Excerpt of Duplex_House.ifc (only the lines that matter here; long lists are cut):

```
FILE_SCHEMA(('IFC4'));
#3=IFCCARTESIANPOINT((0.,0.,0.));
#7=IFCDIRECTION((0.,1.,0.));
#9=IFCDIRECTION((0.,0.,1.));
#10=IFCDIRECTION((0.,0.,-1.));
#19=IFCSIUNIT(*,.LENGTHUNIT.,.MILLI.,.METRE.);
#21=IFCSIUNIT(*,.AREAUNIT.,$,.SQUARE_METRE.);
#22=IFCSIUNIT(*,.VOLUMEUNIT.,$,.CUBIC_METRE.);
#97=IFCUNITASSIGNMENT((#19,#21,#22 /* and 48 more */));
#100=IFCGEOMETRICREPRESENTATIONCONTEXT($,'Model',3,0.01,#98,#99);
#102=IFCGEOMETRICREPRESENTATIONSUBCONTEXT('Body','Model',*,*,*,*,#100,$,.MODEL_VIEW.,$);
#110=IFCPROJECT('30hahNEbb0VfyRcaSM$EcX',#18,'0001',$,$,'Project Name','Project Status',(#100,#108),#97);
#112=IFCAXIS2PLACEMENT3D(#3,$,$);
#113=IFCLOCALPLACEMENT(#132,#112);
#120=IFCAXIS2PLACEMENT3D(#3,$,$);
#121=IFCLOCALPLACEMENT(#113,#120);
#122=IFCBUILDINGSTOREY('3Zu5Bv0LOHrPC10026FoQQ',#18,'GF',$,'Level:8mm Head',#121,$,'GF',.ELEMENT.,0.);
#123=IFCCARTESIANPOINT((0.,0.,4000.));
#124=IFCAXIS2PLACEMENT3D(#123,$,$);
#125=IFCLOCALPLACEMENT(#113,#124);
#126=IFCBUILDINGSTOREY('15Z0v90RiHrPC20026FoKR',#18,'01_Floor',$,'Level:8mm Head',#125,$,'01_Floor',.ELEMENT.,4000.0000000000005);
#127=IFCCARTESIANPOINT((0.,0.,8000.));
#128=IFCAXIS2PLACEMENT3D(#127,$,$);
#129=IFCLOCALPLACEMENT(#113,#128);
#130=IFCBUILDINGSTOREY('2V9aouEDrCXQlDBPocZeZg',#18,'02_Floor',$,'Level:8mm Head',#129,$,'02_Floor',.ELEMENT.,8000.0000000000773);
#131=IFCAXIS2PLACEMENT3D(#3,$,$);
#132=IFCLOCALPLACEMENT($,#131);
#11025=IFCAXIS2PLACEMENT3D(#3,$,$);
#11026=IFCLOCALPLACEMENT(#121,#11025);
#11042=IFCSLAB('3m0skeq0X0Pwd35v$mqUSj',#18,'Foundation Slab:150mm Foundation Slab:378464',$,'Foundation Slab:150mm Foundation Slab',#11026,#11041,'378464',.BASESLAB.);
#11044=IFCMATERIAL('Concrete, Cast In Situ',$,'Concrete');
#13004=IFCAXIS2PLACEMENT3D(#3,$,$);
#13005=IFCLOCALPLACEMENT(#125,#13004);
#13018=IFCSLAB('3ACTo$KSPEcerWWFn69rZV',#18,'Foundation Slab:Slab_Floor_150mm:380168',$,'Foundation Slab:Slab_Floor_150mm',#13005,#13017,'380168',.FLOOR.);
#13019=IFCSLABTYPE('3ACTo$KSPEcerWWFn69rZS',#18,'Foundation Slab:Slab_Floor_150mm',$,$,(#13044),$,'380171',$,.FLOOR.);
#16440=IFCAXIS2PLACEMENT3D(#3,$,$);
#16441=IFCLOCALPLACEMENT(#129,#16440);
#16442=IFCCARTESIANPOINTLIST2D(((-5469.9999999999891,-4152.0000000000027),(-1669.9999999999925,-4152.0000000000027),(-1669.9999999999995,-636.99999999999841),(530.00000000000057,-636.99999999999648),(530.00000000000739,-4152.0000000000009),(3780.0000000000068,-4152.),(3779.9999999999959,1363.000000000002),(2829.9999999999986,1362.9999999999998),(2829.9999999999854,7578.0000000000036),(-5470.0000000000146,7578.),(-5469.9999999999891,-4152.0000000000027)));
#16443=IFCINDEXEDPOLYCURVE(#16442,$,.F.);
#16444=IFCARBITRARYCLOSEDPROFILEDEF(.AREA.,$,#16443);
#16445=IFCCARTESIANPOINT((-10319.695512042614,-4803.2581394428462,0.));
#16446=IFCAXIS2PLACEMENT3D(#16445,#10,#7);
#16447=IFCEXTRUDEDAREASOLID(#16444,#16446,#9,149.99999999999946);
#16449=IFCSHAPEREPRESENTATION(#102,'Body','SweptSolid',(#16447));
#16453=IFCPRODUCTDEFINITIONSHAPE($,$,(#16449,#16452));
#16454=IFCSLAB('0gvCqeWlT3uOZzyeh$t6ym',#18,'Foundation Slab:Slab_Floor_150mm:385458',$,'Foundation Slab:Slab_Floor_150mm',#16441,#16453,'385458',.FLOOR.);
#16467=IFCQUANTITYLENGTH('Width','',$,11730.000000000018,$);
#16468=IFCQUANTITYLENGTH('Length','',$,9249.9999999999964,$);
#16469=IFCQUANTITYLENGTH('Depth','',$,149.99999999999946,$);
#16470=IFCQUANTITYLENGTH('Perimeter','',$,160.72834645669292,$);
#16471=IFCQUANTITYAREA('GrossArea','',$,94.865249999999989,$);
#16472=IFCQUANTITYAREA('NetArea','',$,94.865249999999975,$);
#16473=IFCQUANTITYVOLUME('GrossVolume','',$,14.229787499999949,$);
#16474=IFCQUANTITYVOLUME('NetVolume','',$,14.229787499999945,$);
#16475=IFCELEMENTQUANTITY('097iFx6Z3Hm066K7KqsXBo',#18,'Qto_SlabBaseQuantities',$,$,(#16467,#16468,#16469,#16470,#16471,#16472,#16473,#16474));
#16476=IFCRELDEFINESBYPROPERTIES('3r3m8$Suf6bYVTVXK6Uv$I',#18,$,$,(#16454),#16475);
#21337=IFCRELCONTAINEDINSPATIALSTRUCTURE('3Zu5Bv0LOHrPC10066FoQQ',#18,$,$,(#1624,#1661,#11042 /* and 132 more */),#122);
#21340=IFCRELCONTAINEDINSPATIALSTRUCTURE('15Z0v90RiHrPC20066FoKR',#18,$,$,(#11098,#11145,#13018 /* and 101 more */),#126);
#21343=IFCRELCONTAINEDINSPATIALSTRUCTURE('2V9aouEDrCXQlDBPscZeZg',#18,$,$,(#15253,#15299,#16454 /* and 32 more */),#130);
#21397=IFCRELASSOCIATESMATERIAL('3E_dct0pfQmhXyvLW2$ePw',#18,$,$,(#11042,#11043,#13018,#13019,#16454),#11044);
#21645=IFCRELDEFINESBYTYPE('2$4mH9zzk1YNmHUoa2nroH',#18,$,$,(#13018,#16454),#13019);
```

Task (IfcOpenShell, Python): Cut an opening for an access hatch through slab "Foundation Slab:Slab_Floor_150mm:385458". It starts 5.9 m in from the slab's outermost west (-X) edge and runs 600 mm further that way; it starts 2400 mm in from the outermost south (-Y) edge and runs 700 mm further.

```python
import numpy as np
import ifcopenshell
import ifcopenshell.api.feature
import ifcopenshell.api.geometry
import ifcopenshell.api.pset
import ifcopenshell.api.root
import ifcopenshell.geom
import ifcopenshell.util.element
import ifcopenshell.util.placement
import ifcopenshell.util.representation
import ifcopenshell.util.shape
import ifcopenshell.util.unit

model = ifcopenshell.open("Duplex_House.ifc")
unit_scale = ifcopenshell.util.unit.calculate_unit_scale(model)
area_scale = ifcopenshell.util.unit.calculate_unit_scale(model, "AREAUNIT")
volume_scale = ifcopenshell.util.unit.calculate_unit_scale(model, "VOLUMEUNIT")
settings = ifcopenshell.geom.settings()


def volume(element):
    """Net volume in cubic metres, openings subtracted."""
    shape = ifcopenshell.geom.create_shape(settings, element)
    return ifcopenshell.util.shape.get_volume(shape.geometry)


slab = model.by_guid("0gvCqeWlT3uOZzyeh$t6ym")
before = volume(slab)

# Extent in the slab's own axes, in metres. The edges named are its -X and -Y sides.
slab_shape = ifcopenshell.geom.create_shape(settings, slab)
vertices = ifcopenshell.util.shape.get_vertices(slab_shape.geometry)
x_min, y_min, bottom = vertices.min(axis=0)
top = vertices[:, 2].max()

opening = ifcopenshell.api.root.create_entity(model, ifc_class="IfcOpeningElement", name="Access hatch opening", predefined_type="OPENING")
context = ifcopenshell.util.representation.get_context(model, "Model", "Body", "MODEL_VIEW")
width, depth = 0.6, 0.7
outline = [(0.0, 0.0), (width, 0.0), (width, depth), (0.0, depth), (0.0, 0.0)]
# Overshoot both faces by 50 mm so the cut is clean.
shape = ifcopenshell.api.geometry.add_slab_representation(
    model, context=context, depth=top - bottom + 0.1, polyline=outline
)
ifcopenshell.api.geometry.assign_representation(model, product=opening, representation=shape)

matrix = ifcopenshell.util.placement.get_local_placement(slab.ObjectPlacement)
matrix[:, 3] = matrix @ np.append(np.array([x_min + 5.9, y_min + 2.4, bottom - 0.05]) / unit_scale, 1.0)
ifcopenshell.api.geometry.edit_object_placement(model, product=opening, matrix=matrix, is_si=False)
ifcopenshell.api.feature.add_feature(model, feature=opening, element=slab)

after = volume(slab)

# Update the slab's stored quantities.
qto = model.by_id(ifcopenshell.util.element.get_pset(slab, "Qto_SlabBaseQuantities", should_inherit=False)["id"])
ifcopenshell.api.pset.edit_qto(model, qto=qto, properties={
    "NetArea": after / (top - bottom) / area_scale,
    "NetVolume": after / volume_scale,
})

print(f"slab volume {before:.3f} -> {after:.3f} m3")

model.write("Duplex_House_rev.ifc")
```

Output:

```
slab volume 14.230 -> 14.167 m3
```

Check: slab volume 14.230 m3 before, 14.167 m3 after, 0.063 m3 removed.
